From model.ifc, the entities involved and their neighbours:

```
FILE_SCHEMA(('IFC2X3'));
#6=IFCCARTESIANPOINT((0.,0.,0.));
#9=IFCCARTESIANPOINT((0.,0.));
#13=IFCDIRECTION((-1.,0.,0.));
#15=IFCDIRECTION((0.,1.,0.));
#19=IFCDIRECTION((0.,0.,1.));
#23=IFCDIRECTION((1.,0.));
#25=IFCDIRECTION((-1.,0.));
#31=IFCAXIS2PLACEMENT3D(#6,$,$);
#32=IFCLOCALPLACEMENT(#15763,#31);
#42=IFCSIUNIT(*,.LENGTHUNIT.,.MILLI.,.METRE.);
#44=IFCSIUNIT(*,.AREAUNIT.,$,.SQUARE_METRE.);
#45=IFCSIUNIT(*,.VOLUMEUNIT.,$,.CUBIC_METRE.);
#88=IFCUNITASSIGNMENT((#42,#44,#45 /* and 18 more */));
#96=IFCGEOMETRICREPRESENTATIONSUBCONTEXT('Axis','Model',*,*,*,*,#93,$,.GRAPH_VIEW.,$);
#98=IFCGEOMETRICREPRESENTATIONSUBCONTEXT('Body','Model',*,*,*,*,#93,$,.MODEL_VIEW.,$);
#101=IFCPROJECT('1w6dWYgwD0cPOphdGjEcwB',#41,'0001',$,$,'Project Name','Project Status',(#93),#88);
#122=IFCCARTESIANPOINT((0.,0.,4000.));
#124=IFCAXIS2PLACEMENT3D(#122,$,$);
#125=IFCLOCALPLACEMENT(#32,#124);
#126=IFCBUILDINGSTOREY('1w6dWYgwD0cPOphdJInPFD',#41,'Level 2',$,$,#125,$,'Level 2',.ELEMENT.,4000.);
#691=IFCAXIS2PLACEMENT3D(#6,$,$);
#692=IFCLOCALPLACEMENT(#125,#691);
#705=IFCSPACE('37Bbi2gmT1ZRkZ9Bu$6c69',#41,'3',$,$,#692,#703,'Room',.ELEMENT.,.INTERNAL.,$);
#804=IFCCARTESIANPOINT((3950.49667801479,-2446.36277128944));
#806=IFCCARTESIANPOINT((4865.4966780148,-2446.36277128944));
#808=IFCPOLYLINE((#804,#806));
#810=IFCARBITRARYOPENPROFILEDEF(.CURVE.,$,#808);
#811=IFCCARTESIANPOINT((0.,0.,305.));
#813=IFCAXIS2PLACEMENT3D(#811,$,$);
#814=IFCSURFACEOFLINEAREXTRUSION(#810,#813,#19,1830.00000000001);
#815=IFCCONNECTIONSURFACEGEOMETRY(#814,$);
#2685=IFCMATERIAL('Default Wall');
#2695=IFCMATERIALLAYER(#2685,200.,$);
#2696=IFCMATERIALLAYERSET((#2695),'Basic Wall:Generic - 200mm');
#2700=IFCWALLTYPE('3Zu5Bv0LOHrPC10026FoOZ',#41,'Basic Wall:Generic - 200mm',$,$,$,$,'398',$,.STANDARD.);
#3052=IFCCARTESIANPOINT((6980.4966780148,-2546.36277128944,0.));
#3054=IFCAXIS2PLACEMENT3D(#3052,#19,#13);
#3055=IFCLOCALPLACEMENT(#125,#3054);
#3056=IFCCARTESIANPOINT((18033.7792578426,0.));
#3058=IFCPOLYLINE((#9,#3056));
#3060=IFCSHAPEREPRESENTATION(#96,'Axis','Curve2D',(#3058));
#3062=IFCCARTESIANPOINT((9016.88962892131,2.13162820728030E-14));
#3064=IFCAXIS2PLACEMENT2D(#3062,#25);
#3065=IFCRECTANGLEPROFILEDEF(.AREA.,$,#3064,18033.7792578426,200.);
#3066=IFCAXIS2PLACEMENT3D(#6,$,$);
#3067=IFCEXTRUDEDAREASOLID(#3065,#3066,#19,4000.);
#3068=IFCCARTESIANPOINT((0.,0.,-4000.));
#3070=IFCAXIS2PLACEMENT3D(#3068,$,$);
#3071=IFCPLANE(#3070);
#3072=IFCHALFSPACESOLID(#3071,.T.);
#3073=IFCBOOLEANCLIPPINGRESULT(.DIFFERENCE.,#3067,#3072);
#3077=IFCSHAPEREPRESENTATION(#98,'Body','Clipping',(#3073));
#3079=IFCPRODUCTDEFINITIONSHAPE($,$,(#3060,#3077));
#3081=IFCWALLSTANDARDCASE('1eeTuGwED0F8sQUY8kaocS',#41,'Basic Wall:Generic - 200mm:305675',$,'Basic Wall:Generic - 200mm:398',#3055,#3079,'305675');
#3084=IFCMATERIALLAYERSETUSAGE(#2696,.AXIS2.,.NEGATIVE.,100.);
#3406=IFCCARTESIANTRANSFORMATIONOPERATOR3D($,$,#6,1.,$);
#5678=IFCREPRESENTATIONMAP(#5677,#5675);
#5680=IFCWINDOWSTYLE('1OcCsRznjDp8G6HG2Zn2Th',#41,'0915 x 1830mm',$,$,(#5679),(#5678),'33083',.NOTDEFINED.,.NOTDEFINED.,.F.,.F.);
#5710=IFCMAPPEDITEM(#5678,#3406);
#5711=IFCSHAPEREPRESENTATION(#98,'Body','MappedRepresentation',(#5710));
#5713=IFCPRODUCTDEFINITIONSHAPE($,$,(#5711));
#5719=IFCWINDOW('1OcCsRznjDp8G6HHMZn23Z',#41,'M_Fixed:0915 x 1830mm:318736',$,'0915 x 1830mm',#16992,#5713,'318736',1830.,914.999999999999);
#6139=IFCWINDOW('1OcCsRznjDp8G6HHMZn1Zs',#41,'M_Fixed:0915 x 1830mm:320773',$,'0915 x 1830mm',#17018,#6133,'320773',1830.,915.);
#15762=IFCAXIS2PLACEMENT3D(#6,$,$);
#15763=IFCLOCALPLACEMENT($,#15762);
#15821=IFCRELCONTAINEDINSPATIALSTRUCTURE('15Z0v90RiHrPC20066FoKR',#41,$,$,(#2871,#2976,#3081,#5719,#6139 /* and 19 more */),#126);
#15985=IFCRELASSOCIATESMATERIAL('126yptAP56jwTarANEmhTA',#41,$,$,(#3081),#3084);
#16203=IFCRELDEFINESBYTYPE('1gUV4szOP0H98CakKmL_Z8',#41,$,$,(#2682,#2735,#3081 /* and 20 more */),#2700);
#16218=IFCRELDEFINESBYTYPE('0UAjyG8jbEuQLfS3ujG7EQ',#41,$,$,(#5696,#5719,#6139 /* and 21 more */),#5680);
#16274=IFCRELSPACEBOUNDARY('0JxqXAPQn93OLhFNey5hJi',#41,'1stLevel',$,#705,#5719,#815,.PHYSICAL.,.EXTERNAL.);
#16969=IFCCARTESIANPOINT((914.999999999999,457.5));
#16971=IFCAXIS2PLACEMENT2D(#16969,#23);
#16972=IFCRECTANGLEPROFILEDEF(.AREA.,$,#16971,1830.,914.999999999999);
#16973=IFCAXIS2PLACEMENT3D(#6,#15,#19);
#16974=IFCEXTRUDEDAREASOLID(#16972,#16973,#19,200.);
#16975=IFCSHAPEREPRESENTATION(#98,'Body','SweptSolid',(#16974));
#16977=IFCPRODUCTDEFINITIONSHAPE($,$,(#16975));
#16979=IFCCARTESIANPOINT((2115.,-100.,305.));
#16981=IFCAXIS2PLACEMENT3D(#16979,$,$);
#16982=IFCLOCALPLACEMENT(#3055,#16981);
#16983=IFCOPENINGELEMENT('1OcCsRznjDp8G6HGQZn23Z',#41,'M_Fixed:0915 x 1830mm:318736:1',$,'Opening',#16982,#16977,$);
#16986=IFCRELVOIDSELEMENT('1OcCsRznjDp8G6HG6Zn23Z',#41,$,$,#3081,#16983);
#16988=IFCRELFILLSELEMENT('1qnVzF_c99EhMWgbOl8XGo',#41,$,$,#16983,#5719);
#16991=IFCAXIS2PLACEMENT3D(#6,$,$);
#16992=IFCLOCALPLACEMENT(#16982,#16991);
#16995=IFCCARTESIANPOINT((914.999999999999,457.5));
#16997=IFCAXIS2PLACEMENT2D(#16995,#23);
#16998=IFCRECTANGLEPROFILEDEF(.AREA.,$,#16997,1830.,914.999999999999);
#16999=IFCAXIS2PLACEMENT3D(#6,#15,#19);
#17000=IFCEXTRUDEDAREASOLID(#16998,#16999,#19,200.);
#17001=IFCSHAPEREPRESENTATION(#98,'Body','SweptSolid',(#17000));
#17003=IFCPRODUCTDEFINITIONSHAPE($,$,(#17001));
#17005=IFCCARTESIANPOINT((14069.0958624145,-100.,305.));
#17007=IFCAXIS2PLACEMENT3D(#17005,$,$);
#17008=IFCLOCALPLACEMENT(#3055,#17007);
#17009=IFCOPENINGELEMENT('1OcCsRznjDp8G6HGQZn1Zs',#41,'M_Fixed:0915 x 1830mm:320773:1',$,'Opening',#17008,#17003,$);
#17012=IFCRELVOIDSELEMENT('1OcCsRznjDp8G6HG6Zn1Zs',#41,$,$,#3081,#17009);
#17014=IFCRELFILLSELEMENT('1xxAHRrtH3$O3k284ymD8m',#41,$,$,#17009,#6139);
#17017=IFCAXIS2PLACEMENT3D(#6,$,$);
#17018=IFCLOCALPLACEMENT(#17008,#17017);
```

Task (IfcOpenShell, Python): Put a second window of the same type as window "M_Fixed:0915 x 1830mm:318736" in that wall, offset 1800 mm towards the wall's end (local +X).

```python
import numpy as np
import ifcopenshell
import ifcopenshell.api.feature
import ifcopenshell.api.geometry
import ifcopenshell.api.root
import ifcopenshell.geom
import ifcopenshell.util.element
import ifcopenshell.util.placement
import ifcopenshell.util.shape
import ifcopenshell.util.unit

model = ifcopenshell.open("model.ifc")
unit_scale = ifcopenshell.util.unit.calculate_unit_scale(model)
settings = ifcopenshell.geom.settings()


def volume(element):
    """Net volume in cubic metres, openings subtracted."""
    shape = ifcopenshell.geom.create_shape(settings, element)
    return ifcopenshell.util.shape.get_volume(shape.geometry)


def reuse_history(source, copy):
    """copy_class also copies each property set's owner history, people and application; keep the originals."""
    for rel in copy.IsDefinedBy:
        if rel.is_a("IfcRelDefinesByProperties") and (history := rel.RelatingPropertyDefinition.OwnerHistory):
            rel.RelatingPropertyDefinition.OwnerHistory = source.OwnerHistory
            ifcopenshell.util.element.remove_deep2(model, history)


window = model.by_guid("1OcCsRznjDp8G6HHMZn23Z")
opening = window.FillsVoids[0].RelatingOpeningElement
wall = opening.VoidsElements[0].RelatingBuildingElement
before = volume(wall)
shift = ifcopenshell.util.placement.get_local_placement(wall.ObjectPlacement)[:3, 0] * 1.8 / unit_scale

# copy_class copies the void relationship, type, container and properties, but no geometry.
new_opening = ifcopenshell.api.root.copy_class(model, product=opening)
new_opening.Representation = ifcopenshell.util.element.copy_deep(
    model, opening.Representation, exclude=["IfcGeometricRepresentationContext", "IfcRepresentationMap"]
)
new_opening.Name = "M_Fixed:0915 x 1830mm"
new_window = ifcopenshell.api.root.copy_class(model, product=window)
new_window.Representation = ifcopenshell.util.element.copy_deep(
    model, window.Representation, exclude=["IfcGeometricRepresentationContext", "IfcRepresentationMap"]
)
new_window.Name = "M_Fixed:0915 x 1830mm"
new_window.Tag = None
reuse_history(window, new_window)
fills = ifcopenshell.api.feature.add_filling(model, opening=new_opening, element=new_window)
fills.OwnerHistory = new_window.OwnerHistory  # required in IFC2X3

for old, new in ((opening, new_opening), (window, new_window)):
    matrix = ifcopenshell.util.placement.get_local_placement(old.ObjectPlacement)
    matrix[:3, 3] += shift
    ifcopenshell.api.geometry.edit_object_placement(model, product=new, matrix=matrix, is_si=False)

# The copied space boundaries still share their surfaces with the original.
for rel in new_window.ProvidesBoundaries:
    if rel.ConnectionGeometry:
        rel.ConnectionGeometry = ifcopenshell.util.element.copy_deep(model, rel.ConnectionGeometry)

# Space boundary surfaces are stored in each space's coordinates; move them too.
for rel in new_window.ProvidesBoundaries:
    if not rel.ConnectionGeometry:
        continue
    surface = rel.ConnectionGeometry.SurfaceOnRelatingElement
    space_matrix = ifcopenshell.util.placement.get_local_placement(rel.RelatingSpace.ObjectPlacement)
    point = np.array(surface.Position.Location.Coordinates) + space_matrix[:3, :3].T @ shift
    surface.Position = model.createIfcAxis2Placement3D(
        model.createIfcCartesianPoint(point.tolist()), surface.Position.Axis, surface.Position.RefDirection
    )

after = volume(wall)

print(f"wall volume {before:.3f} -> {after:.3f} m3")

model.write("model_edited.ifc")
```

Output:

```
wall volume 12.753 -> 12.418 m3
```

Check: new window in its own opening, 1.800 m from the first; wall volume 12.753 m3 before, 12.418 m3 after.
